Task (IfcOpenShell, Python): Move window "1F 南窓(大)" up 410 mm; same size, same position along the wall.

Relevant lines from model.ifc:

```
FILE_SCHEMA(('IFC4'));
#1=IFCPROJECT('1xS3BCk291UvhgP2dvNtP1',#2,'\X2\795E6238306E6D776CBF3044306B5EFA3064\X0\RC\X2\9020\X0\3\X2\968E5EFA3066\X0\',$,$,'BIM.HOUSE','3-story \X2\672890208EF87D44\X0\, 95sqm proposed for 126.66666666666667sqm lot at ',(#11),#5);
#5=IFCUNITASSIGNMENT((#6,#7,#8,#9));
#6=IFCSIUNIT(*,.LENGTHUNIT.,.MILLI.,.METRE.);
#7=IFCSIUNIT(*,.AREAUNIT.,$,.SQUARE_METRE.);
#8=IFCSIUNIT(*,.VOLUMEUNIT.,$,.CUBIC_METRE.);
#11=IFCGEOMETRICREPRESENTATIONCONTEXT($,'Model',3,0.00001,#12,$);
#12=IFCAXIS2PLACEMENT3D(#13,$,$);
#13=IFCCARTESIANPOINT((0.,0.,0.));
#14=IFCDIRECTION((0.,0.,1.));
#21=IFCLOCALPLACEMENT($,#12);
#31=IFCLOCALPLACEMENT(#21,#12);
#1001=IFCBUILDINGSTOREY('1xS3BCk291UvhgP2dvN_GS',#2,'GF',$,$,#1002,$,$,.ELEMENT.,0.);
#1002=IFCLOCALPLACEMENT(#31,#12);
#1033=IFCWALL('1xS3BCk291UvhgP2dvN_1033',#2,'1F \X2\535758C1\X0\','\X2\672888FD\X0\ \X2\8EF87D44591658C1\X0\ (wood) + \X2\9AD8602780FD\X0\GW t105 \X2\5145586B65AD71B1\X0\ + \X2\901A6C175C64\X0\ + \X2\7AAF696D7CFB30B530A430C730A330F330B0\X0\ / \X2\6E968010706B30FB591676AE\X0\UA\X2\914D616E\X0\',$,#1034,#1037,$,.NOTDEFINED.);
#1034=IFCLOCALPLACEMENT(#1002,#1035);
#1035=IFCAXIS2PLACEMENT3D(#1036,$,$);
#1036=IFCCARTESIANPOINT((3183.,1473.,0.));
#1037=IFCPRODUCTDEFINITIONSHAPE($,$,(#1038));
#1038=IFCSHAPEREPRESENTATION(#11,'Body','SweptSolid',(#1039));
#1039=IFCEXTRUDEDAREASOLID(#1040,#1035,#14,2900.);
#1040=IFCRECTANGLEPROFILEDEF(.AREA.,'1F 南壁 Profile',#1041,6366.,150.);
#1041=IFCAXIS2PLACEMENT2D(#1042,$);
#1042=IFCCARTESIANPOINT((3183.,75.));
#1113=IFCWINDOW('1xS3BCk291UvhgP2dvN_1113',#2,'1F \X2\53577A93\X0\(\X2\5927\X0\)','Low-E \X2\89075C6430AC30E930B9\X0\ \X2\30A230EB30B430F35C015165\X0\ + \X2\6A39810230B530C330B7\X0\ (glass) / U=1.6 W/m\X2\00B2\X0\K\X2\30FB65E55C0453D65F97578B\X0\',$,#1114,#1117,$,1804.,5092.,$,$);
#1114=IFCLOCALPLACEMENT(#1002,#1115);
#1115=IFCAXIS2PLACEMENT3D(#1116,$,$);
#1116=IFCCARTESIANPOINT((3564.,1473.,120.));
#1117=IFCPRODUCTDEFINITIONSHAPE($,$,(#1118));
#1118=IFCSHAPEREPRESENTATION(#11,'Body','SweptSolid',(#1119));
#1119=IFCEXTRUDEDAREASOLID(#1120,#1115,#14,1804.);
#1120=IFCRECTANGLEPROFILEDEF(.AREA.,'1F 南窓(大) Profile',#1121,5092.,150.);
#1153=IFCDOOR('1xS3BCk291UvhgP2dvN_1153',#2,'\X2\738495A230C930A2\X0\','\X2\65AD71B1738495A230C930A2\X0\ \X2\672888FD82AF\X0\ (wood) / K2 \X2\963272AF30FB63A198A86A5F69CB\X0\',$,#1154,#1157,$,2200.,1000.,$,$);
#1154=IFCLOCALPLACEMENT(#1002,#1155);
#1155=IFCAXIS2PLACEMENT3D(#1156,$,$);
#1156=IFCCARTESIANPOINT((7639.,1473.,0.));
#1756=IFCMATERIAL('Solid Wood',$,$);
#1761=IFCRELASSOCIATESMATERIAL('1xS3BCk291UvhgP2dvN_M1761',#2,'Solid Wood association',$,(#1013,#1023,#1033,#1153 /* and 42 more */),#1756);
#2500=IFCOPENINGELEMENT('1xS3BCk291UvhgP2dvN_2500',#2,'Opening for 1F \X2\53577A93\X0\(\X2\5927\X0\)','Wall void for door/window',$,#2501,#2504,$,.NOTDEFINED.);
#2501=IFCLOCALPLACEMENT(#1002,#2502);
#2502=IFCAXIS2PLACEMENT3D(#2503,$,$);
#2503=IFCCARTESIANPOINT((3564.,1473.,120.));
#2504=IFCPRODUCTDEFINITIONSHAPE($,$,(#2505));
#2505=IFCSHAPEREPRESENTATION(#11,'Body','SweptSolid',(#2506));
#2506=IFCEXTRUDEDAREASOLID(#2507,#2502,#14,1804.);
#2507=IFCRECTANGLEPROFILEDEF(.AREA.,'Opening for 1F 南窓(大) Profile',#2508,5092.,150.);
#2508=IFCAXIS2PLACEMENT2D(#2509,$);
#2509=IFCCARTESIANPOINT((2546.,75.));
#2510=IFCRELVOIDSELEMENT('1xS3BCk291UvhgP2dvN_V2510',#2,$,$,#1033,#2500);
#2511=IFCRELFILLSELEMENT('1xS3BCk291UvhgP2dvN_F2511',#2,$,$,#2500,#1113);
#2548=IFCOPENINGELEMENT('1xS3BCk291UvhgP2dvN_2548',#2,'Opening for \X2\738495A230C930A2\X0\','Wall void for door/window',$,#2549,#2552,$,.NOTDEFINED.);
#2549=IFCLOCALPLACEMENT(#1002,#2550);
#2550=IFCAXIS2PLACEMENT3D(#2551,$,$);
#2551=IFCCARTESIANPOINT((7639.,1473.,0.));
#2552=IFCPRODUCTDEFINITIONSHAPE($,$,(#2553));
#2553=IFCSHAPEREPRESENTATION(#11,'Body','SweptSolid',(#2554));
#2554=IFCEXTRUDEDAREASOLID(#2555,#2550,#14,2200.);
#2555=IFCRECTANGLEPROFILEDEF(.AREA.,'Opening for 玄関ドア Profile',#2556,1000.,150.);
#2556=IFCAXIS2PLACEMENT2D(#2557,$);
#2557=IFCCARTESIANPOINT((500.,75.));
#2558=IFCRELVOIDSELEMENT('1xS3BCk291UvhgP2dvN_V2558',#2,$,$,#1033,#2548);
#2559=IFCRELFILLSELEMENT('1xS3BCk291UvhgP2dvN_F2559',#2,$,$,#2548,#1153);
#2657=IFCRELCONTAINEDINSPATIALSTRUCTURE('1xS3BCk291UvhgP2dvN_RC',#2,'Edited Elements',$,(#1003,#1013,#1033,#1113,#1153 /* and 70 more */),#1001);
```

```python
import numpy as np
import ifcopenshell
import ifcopenshell.api.geometry
import ifcopenshell.util.placement
import ifcopenshell.util.unit

model = ifcopenshell.open("model.ifc")
unit_scale = ifcopenshell.util.unit.calculate_unit_scale(model)

window = model.by_guid("1xS3BCk291UvhgP2dvN_1113")
opening = window.FillsVoids[0].RelatingOpeningElement
dz = 410.0

shift = np.array([0.0, 0.0, dz])
# The window is not placed relative to its opening, so move both.
for product in (opening, window):
    matrix = ifcopenshell.util.placement.get_local_placement(product.ObjectPlacement)
    matrix[:3, 3] += shift
    ifcopenshell.api.geometry.edit_object_placement(model, product=product, matrix=matrix, is_si=False)

print(f"moved by {dz * unit_scale:+.3f} m")

model.write("model_edited.ifc")
```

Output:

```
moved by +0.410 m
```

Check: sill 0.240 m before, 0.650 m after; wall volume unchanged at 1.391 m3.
